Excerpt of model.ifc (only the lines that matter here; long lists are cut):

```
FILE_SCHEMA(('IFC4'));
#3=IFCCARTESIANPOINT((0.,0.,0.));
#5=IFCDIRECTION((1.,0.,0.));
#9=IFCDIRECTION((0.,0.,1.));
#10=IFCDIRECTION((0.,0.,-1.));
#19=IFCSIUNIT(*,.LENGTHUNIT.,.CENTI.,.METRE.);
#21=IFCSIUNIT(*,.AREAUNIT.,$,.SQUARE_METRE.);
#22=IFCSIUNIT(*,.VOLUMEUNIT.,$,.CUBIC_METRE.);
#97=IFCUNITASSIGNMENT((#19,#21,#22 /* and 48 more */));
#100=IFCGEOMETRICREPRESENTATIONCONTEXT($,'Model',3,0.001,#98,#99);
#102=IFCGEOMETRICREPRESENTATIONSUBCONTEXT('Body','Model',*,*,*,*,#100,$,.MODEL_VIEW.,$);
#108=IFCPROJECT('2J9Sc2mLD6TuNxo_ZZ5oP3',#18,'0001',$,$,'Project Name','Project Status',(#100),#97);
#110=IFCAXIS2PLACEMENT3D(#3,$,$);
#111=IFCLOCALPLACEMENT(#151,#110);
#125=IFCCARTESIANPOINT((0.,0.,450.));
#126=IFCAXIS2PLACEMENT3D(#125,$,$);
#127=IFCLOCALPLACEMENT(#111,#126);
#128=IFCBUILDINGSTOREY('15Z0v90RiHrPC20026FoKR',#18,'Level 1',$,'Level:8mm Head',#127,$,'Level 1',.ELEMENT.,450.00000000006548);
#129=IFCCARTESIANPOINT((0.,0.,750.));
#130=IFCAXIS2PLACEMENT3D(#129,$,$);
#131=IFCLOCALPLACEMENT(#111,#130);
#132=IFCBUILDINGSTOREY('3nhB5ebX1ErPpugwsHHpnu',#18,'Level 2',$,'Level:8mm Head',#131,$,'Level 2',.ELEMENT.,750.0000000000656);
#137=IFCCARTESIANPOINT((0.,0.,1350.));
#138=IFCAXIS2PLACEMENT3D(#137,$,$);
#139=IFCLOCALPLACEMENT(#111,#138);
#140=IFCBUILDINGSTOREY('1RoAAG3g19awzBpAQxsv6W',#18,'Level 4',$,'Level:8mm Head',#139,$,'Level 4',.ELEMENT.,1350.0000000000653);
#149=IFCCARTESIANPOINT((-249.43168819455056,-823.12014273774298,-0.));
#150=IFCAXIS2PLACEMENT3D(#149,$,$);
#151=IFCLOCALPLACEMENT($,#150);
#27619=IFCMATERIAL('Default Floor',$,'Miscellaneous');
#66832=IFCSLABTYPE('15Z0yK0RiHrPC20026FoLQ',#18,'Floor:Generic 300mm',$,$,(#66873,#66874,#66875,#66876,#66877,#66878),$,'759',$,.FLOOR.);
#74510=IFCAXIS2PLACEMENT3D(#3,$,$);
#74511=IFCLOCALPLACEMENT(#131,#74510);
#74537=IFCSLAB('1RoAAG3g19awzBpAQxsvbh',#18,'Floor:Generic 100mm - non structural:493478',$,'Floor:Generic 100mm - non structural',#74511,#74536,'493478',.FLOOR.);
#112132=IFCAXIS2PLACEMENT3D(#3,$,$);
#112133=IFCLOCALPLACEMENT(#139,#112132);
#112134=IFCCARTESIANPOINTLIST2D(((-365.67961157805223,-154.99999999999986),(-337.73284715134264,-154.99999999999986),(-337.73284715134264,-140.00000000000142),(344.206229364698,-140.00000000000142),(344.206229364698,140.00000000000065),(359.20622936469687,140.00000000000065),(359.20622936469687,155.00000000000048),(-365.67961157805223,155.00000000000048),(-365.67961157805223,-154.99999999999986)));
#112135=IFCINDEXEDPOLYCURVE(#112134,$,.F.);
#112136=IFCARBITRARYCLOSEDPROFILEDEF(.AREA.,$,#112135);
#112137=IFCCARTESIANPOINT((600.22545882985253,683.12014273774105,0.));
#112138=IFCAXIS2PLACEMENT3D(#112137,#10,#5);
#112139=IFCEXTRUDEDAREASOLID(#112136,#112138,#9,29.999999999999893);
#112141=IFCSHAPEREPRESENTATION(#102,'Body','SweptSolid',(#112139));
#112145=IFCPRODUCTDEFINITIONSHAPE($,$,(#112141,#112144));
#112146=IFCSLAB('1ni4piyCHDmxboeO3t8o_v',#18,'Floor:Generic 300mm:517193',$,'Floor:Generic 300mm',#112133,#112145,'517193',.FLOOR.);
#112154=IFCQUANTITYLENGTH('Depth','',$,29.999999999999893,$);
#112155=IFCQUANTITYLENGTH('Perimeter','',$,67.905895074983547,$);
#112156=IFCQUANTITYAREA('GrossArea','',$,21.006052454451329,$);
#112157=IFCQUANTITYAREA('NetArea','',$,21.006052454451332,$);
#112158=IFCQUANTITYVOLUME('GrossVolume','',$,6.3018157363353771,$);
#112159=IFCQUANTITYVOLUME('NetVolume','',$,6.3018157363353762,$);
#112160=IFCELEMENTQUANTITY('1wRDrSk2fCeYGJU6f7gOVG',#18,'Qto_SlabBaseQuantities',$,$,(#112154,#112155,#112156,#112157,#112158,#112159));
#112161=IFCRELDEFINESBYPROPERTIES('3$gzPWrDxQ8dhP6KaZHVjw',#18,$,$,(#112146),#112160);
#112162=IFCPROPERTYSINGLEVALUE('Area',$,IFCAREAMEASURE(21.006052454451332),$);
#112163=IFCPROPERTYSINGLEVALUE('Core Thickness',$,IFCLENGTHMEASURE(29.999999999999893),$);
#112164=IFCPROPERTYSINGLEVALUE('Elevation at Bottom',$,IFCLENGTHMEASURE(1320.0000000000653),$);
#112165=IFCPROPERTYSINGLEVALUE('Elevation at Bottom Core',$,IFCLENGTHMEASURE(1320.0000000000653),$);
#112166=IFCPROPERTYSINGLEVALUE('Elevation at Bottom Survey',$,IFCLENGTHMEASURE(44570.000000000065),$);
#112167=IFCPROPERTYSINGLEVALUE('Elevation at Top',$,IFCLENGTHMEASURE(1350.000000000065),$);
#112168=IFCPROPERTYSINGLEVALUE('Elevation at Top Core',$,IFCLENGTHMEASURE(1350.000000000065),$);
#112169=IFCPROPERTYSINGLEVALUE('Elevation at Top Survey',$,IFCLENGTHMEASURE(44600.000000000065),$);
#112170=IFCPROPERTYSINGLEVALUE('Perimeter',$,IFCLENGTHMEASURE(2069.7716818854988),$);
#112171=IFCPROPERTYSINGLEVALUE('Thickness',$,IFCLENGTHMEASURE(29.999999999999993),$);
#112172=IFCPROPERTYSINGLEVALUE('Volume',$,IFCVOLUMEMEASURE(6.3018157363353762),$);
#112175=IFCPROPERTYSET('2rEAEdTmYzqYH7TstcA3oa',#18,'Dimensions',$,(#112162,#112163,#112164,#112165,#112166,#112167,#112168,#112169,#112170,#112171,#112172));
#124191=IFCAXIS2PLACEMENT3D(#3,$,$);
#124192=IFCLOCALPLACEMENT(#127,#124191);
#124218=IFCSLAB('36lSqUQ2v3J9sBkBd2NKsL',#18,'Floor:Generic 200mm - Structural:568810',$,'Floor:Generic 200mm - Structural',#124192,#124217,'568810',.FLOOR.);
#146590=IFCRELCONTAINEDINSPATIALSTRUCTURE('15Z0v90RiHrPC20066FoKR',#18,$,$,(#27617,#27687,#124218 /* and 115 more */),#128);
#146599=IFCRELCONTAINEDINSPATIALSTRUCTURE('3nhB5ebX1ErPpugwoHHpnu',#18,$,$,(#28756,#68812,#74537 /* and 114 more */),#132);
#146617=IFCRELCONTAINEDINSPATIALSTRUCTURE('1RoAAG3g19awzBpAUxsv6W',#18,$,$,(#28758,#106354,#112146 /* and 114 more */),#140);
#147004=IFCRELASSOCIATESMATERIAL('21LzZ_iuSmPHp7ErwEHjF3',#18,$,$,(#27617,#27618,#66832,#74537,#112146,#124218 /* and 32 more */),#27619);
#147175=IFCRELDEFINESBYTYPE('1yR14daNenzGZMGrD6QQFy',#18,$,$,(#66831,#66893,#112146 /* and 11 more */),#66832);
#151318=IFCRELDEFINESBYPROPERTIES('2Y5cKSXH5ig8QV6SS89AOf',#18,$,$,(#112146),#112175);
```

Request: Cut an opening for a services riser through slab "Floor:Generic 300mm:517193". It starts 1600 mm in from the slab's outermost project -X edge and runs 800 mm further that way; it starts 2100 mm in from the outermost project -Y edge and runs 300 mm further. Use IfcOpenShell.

```python
import numpy as np
import ifcopenshell
import ifcopenshell.api.feature
import ifcopenshell.api.geometry
import ifcopenshell.api.pset
import ifcopenshell.api.root
import ifcopenshell.geom
import ifcopenshell.util.element
import ifcopenshell.util.placement
import ifcopenshell.util.representation
import ifcopenshell.util.shape
import ifcopenshell.util.unit

model = ifcopenshell.open("model.ifc")
unit_scale = ifcopenshell.util.unit.calculate_unit_scale(model)
area_scale = ifcopenshell.util.unit.calculate_unit_scale(model, "AREAUNIT")
volume_scale = ifcopenshell.util.unit.calculate_unit_scale(model, "VOLUMEUNIT")
settings = ifcopenshell.geom.settings()


def volume(element):
    """Net volume in cubic metres, openings subtracted."""
    shape = ifcopenshell.geom.create_shape(settings, element)
    return ifcopenshell.util.shape.get_volume(shape.geometry)


slab = model.by_id(112146)
before = volume(slab)

# Extent in the slab's own axes, in metres. The edges named are its -X and -Y sides.
slab_shape = ifcopenshell.geom.create_shape(settings, slab)
vertices = ifcopenshell.util.shape.get_vertices(slab_shape.geometry)
x_min, y_min, bottom = vertices.min(axis=0)
top = vertices[:, 2].max()

opening = ifcopenshell.api.root.create_entity(model, ifc_class="IfcOpeningElement", name="Services riser opening", predefined_type="OPENING")
context = ifcopenshell.util.representation.get_context(model, "Model", "Body", "MODEL_VIEW")
width, depth = 0.8, 0.3
outline = [(0.0, 0.0), (width, 0.0), (width, depth), (0.0, depth), (0.0, 0.0)]
# Overshoot both faces by 50 mm so the cut is clean.
shape = ifcopenshell.api.geometry.add_slab_representation(
    model, context=context, depth=top - bottom + 0.1, polyline=outline
)
ifcopenshell.api.geometry.assign_representation(model, product=opening, representation=shape)

matrix = ifcopenshell.util.placement.get_local_placement(slab.ObjectPlacement)
matrix[:, 3] = matrix @ np.append(np.array([x_min + 1.6, y_min + 2.1, bottom - 0.05]) / unit_scale, 1.0)
ifcopenshell.api.geometry.edit_object_placement(model, product=opening, matrix=matrix, is_si=False)
ifcopenshell.api.feature.add_feature(model, feature=opening, element=slab)

after = volume(slab)

# Update the slab's stored quantities.
qto = model.by_id(ifcopenshell.util.element.get_pset(slab, "Qto_SlabBaseQuantities", should_inherit=False)["id"])
ifcopenshell.api.pset.edit_qto(model, qto=qto, properties={
    "NetArea": after / (top - bottom) / area_scale,
    "NetVolume": after / volume_scale,
})
pset = model.by_id(ifcopenshell.util.element.get_pset(slab, "Dimensions", should_inherit=False)["id"])
ifcopenshell.api.pset.edit_pset(model, pset=pset, properties={
    "Area": model.create_entity("IfcAreaMeasure", after / (top - bottom) / area_scale),
    "Volume": model.create_entity("IfcVolumeMeasure", after / volume_scale),
})

print(f"slab volume {before:.3f} -> {after:.3f} m3")

model.write("model-out.ifc")
```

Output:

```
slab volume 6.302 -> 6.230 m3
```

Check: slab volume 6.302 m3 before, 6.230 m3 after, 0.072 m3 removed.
